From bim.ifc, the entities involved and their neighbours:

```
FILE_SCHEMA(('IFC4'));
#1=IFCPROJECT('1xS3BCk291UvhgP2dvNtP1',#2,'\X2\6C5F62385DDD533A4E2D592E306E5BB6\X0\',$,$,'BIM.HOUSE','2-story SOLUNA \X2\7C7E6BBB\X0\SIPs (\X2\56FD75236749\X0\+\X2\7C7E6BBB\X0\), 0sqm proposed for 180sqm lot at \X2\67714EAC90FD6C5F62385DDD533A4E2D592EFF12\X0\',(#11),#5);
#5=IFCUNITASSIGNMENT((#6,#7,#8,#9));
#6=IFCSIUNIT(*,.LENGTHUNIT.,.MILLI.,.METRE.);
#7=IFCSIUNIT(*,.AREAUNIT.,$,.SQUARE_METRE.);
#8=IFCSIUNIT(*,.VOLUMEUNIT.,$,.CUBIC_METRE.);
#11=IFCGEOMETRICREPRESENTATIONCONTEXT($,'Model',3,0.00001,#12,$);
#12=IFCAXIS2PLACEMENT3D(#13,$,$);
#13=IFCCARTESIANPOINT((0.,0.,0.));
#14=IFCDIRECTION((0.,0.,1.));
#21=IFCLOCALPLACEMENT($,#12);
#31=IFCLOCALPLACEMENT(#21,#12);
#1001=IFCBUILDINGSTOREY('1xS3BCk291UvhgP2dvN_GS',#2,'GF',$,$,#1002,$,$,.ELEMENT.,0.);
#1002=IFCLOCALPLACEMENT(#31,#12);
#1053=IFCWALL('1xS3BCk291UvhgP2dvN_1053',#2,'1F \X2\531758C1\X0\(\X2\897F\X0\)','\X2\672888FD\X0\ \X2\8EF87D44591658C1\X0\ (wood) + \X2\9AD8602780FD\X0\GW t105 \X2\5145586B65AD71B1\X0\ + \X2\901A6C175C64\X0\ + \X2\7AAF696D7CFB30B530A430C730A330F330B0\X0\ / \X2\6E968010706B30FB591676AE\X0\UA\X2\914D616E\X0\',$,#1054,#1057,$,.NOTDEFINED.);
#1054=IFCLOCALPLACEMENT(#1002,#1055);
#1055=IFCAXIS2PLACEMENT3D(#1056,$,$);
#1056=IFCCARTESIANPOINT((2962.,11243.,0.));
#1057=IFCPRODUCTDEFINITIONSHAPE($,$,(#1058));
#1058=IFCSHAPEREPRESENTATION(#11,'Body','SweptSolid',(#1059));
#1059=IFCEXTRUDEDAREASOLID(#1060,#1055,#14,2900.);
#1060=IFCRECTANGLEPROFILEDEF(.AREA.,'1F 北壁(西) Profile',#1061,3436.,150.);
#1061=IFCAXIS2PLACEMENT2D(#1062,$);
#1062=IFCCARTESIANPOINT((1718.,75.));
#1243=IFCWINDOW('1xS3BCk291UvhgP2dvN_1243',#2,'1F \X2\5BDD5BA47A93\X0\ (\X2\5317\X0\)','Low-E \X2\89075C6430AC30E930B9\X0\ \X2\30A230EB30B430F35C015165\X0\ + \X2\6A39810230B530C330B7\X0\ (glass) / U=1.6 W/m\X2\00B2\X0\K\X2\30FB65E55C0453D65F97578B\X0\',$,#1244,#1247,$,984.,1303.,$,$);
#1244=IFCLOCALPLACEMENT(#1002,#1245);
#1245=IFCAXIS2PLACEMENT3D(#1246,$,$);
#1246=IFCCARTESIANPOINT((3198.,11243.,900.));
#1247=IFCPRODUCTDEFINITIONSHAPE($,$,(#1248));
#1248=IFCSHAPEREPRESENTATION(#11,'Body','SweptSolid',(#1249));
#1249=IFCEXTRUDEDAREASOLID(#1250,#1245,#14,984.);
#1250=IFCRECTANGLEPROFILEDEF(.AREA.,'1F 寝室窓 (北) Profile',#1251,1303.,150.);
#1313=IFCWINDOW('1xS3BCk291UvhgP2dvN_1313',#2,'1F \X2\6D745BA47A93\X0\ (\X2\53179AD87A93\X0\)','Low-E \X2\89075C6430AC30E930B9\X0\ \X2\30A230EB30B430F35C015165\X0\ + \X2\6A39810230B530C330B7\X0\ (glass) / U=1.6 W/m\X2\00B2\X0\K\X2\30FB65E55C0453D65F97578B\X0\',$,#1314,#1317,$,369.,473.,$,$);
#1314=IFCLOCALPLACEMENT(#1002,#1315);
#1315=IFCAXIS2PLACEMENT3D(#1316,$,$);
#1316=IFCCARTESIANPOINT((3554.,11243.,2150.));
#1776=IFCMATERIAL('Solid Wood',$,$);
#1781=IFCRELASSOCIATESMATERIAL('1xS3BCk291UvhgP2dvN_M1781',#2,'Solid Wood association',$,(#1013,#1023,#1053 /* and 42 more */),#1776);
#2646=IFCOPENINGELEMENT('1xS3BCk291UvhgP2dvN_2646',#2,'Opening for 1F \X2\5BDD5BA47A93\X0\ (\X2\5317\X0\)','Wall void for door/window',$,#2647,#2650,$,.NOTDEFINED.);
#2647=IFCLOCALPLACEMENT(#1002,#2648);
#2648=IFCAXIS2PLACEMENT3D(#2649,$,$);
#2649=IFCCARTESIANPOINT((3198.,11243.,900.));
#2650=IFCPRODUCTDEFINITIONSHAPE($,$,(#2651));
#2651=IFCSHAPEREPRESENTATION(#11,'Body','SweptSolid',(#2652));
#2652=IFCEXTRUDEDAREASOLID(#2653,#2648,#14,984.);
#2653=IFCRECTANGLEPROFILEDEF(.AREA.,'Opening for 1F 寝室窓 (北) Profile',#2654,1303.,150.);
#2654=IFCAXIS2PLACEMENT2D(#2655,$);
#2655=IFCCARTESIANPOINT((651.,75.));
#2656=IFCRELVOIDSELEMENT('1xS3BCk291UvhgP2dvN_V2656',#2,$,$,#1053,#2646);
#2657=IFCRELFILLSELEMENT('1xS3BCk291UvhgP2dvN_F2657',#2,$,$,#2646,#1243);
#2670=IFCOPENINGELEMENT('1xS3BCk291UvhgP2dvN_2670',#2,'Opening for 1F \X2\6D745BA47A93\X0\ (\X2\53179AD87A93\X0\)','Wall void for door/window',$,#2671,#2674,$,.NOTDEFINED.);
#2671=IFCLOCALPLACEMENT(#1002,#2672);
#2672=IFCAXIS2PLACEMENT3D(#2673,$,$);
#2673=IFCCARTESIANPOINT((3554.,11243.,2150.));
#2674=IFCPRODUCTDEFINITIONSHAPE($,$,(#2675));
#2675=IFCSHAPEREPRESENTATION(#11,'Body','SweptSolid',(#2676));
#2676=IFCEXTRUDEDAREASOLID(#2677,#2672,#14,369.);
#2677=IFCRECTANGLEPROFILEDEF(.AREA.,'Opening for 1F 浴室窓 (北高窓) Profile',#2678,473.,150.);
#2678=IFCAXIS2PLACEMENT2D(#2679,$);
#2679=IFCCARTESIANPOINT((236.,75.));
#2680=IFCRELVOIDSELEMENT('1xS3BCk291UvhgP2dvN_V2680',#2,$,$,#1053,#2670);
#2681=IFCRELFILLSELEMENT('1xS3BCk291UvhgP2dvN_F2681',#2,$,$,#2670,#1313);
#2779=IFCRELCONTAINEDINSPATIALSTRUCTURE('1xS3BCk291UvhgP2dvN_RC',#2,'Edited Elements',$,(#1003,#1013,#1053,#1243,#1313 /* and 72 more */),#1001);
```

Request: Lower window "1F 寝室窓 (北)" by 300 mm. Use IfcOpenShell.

```python
import numpy as np
import ifcopenshell
import ifcopenshell.api.geometry
import ifcopenshell.util.placement
import ifcopenshell.util.unit

model = ifcopenshell.open("bim.ifc")
unit_scale = ifcopenshell.util.unit.calculate_unit_scale(model)

window = model.by_id(1243)
opening = window.FillsVoids[0].RelatingOpeningElement
dz = -0.3 / unit_scale

shift = np.array([0.0, 0.0, dz])
# The window is not placed relative to its opening, so move both.
for product in (opening, window):
    matrix = ifcopenshell.util.placement.get_local_placement(product.ObjectPlacement)
    matrix[:3, 3] += shift
    ifcopenshell.api.geometry.edit_object_placement(model, product=product, matrix=matrix, is_si=False)

print(f"moved by {dz * unit_scale:+.3f} m")

model.write("bim_edited.ifc")
```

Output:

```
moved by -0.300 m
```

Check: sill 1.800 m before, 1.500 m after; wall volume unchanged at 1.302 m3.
